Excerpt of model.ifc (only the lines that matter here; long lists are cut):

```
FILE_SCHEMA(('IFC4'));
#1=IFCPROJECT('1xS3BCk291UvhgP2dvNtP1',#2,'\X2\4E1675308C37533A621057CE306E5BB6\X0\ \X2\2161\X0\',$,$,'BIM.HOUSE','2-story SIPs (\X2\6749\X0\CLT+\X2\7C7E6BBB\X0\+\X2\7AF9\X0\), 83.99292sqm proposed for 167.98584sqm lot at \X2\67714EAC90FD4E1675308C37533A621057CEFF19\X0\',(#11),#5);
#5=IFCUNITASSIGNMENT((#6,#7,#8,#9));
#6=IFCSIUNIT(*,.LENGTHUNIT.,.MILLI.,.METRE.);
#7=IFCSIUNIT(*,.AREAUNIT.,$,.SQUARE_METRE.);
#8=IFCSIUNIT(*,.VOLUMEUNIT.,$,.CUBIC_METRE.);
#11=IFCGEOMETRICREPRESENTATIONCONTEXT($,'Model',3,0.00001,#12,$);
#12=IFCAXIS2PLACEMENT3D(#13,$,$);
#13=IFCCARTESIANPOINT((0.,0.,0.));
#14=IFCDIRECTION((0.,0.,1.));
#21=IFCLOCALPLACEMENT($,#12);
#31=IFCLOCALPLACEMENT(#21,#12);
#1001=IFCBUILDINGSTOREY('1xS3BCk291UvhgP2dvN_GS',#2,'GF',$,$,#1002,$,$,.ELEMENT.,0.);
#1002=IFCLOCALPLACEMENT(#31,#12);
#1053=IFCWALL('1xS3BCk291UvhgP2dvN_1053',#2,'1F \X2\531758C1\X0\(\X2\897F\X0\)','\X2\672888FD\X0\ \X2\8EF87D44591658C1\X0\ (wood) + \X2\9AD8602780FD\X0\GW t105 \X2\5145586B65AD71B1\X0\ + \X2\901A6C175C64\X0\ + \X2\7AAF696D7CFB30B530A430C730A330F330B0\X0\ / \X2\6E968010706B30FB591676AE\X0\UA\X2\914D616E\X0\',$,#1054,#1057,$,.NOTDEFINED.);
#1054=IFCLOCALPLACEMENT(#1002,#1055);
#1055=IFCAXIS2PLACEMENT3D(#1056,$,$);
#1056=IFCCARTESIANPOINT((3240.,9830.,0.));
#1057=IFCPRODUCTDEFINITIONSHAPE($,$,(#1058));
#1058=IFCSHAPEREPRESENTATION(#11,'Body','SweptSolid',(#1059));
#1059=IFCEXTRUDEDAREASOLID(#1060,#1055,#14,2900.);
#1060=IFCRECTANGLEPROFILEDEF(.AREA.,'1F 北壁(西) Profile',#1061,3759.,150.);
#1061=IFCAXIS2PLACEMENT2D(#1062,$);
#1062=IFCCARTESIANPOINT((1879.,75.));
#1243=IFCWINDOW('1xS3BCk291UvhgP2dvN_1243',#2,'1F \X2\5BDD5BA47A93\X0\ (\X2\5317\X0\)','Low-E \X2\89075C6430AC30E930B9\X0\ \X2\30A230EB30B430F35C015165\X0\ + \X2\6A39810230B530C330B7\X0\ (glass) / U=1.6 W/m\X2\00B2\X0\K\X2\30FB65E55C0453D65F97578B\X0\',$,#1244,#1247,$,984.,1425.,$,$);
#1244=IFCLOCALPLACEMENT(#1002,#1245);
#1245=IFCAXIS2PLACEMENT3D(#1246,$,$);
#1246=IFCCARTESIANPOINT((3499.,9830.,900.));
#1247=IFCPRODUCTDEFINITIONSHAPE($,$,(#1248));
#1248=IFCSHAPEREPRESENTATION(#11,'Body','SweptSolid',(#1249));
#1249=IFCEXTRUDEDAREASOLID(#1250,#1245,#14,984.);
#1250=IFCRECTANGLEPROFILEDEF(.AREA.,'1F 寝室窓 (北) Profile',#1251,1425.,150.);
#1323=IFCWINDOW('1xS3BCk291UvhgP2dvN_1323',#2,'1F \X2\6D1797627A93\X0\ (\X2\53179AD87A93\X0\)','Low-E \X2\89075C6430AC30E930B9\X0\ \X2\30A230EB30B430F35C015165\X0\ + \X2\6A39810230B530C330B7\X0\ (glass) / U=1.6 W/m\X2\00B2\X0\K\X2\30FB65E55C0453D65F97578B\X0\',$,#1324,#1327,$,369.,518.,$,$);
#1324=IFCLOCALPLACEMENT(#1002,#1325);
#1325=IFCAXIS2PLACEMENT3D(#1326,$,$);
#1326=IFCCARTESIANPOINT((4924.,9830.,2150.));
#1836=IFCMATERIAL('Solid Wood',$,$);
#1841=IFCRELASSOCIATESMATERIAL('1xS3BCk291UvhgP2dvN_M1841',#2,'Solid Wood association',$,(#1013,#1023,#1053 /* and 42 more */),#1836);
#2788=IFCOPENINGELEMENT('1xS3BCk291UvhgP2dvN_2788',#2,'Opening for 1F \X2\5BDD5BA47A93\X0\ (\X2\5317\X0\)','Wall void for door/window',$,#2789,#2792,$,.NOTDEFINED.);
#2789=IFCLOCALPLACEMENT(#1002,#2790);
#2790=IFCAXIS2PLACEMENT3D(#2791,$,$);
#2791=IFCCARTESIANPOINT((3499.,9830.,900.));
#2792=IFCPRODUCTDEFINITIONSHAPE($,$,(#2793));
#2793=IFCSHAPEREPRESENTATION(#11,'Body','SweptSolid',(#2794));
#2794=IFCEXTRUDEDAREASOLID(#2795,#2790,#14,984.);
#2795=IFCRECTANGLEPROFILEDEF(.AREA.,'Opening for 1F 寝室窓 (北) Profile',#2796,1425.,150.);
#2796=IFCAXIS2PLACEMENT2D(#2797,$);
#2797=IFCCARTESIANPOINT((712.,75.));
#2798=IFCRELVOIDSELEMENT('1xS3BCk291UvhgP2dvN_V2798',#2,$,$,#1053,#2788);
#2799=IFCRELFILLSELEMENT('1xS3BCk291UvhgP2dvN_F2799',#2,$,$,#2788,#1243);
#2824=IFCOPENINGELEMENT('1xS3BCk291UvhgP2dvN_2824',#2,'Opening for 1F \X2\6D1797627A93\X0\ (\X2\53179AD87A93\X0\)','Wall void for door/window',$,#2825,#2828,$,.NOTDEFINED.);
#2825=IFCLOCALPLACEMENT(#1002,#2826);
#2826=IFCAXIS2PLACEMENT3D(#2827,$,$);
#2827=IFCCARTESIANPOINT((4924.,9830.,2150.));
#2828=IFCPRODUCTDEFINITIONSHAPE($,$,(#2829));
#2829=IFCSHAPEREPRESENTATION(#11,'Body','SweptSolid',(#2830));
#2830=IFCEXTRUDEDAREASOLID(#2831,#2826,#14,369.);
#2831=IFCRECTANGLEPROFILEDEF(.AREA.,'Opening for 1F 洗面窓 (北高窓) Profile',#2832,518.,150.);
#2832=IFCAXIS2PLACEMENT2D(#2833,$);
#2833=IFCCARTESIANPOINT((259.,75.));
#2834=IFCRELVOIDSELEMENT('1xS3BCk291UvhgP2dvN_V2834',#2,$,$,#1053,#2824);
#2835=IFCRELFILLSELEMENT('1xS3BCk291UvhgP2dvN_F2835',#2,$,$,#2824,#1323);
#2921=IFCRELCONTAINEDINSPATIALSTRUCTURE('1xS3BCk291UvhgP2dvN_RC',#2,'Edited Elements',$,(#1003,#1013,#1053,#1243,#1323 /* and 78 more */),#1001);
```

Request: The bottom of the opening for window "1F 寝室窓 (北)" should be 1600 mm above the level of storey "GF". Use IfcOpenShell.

```python
import numpy as np
import ifcopenshell
import ifcopenshell.api.geometry
import ifcopenshell.geom
import ifcopenshell.util.element
import ifcopenshell.util.placement
import ifcopenshell.util.shape
import ifcopenshell.util.unit

model = ifcopenshell.open("model.ifc")
unit_scale = ifcopenshell.util.unit.calculate_unit_scale(model)

window = model.by_guid("1xS3BCk291UvhgP2dvN_1243")
opening = window.FillsVoids[0].RelatingOpeningElement
storey = ifcopenshell.util.element.get_container(window, ifc_class="IfcBuildingStorey")
level = ifcopenshell.util.placement.get_local_placement(storey.ObjectPlacement)[2, 3]

# The opening's origin need not be at the sill, so measure its lowest point.
shape = ifcopenshell.geom.create_shape(ifcopenshell.geom.settings(), opening)
bottom = ifcopenshell.util.shape.get_shape_bottom_elevation(shape, shape.geometry) / unit_scale
dz = level + 1.6 / unit_scale - bottom

shift = np.array([0.0, 0.0, dz])
# The window is not placed relative to its opening, so move both.
for product in (opening, window):
    matrix = ifcopenshell.util.placement.get_local_placement(product.ObjectPlacement)
    matrix[:3, 3] += shift
    ifcopenshell.api.geometry.edit_object_placement(model, product=product, matrix=matrix, is_si=False)

print(f"moved by {dz * unit_scale:+.3f} m")

model.write("model-out.ifc")
```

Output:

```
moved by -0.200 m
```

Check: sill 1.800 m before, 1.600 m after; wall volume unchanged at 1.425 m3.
